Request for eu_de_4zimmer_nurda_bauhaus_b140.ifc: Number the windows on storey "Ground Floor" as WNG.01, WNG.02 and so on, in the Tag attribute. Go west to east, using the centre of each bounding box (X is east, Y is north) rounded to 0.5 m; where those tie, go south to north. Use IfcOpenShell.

First a look at what the model holds.

```python
import ifcopenshell
import ifcopenshell.util.element
import ifcopenshell.util.placement

model = ifcopenshell.open("eu_de_4zimmer_nurda_bauhaus_b140.ifc")
print(model.schema)
storey = next(s for s in model.by_type("IfcBuildingStorey") if s.Name == "Ground Floor")
windows = [e for e in ifcopenshell.util.element.get_decomposition(storey) if e.is_a("IfcWindow")]
for e in sorted(windows, key=lambda e: e.id()):
    origin = ifcopenshell.util.placement.get_local_placement(e.ObjectPlacement)[:3, 3]
    print(e.id(), e.Tag, e.Name, origin.round(2) + 0.0, sep=" | ")
```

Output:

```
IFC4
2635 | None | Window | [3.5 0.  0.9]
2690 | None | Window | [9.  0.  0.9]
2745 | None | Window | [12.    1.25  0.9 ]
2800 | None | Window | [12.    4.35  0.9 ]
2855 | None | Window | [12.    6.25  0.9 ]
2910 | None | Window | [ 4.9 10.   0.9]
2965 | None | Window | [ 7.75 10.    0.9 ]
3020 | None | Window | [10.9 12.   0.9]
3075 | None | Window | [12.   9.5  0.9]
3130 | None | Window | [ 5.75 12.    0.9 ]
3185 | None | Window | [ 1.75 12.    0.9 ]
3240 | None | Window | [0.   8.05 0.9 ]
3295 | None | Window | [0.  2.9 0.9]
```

```python
import ifcopenshell
import ifcopenshell.geom
import ifcopenshell.util.element
import ifcopenshell.util.shape

model = ifcopenshell.open("eu_de_4zimmer_nurda_bauhaus_b140.ifc")
settings = ifcopenshell.geom.settings()
settings.set("use-world-coords", True)


def centre(element):
    shape = ifcopenshell.geom.create_shape(settings, element)
    return ifcopenshell.util.shape.get_bbox_centroid(shape.geometry)


storey = next(s for s in model.by_type("IfcBuildingStorey") if s.Name == "Ground Floor")
windows = [e for e in ifcopenshell.util.element.get_decomposition(storey) if e.is_a("IfcWindow")]

# Insertion points can sit at a corner or the storey origin, so sort by the geometry (in metres).
centres = {e: centre(e) for e in windows}
windows.sort(key=lambda e: (round(centres[e][0] / 0.5), centres[e][1]))

for i, e in enumerate(windows, start=1):
    number = f"WNG.{i:02d}"
    e.Tag = number
    print(e.id(), number)

model.write("eu_de_4zimmer_nurda_bauhaus_b140-out.ifc")
```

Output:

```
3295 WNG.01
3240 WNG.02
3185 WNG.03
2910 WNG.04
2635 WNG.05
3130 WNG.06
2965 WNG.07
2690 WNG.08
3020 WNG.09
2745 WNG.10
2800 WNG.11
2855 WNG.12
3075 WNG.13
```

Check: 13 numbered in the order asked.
